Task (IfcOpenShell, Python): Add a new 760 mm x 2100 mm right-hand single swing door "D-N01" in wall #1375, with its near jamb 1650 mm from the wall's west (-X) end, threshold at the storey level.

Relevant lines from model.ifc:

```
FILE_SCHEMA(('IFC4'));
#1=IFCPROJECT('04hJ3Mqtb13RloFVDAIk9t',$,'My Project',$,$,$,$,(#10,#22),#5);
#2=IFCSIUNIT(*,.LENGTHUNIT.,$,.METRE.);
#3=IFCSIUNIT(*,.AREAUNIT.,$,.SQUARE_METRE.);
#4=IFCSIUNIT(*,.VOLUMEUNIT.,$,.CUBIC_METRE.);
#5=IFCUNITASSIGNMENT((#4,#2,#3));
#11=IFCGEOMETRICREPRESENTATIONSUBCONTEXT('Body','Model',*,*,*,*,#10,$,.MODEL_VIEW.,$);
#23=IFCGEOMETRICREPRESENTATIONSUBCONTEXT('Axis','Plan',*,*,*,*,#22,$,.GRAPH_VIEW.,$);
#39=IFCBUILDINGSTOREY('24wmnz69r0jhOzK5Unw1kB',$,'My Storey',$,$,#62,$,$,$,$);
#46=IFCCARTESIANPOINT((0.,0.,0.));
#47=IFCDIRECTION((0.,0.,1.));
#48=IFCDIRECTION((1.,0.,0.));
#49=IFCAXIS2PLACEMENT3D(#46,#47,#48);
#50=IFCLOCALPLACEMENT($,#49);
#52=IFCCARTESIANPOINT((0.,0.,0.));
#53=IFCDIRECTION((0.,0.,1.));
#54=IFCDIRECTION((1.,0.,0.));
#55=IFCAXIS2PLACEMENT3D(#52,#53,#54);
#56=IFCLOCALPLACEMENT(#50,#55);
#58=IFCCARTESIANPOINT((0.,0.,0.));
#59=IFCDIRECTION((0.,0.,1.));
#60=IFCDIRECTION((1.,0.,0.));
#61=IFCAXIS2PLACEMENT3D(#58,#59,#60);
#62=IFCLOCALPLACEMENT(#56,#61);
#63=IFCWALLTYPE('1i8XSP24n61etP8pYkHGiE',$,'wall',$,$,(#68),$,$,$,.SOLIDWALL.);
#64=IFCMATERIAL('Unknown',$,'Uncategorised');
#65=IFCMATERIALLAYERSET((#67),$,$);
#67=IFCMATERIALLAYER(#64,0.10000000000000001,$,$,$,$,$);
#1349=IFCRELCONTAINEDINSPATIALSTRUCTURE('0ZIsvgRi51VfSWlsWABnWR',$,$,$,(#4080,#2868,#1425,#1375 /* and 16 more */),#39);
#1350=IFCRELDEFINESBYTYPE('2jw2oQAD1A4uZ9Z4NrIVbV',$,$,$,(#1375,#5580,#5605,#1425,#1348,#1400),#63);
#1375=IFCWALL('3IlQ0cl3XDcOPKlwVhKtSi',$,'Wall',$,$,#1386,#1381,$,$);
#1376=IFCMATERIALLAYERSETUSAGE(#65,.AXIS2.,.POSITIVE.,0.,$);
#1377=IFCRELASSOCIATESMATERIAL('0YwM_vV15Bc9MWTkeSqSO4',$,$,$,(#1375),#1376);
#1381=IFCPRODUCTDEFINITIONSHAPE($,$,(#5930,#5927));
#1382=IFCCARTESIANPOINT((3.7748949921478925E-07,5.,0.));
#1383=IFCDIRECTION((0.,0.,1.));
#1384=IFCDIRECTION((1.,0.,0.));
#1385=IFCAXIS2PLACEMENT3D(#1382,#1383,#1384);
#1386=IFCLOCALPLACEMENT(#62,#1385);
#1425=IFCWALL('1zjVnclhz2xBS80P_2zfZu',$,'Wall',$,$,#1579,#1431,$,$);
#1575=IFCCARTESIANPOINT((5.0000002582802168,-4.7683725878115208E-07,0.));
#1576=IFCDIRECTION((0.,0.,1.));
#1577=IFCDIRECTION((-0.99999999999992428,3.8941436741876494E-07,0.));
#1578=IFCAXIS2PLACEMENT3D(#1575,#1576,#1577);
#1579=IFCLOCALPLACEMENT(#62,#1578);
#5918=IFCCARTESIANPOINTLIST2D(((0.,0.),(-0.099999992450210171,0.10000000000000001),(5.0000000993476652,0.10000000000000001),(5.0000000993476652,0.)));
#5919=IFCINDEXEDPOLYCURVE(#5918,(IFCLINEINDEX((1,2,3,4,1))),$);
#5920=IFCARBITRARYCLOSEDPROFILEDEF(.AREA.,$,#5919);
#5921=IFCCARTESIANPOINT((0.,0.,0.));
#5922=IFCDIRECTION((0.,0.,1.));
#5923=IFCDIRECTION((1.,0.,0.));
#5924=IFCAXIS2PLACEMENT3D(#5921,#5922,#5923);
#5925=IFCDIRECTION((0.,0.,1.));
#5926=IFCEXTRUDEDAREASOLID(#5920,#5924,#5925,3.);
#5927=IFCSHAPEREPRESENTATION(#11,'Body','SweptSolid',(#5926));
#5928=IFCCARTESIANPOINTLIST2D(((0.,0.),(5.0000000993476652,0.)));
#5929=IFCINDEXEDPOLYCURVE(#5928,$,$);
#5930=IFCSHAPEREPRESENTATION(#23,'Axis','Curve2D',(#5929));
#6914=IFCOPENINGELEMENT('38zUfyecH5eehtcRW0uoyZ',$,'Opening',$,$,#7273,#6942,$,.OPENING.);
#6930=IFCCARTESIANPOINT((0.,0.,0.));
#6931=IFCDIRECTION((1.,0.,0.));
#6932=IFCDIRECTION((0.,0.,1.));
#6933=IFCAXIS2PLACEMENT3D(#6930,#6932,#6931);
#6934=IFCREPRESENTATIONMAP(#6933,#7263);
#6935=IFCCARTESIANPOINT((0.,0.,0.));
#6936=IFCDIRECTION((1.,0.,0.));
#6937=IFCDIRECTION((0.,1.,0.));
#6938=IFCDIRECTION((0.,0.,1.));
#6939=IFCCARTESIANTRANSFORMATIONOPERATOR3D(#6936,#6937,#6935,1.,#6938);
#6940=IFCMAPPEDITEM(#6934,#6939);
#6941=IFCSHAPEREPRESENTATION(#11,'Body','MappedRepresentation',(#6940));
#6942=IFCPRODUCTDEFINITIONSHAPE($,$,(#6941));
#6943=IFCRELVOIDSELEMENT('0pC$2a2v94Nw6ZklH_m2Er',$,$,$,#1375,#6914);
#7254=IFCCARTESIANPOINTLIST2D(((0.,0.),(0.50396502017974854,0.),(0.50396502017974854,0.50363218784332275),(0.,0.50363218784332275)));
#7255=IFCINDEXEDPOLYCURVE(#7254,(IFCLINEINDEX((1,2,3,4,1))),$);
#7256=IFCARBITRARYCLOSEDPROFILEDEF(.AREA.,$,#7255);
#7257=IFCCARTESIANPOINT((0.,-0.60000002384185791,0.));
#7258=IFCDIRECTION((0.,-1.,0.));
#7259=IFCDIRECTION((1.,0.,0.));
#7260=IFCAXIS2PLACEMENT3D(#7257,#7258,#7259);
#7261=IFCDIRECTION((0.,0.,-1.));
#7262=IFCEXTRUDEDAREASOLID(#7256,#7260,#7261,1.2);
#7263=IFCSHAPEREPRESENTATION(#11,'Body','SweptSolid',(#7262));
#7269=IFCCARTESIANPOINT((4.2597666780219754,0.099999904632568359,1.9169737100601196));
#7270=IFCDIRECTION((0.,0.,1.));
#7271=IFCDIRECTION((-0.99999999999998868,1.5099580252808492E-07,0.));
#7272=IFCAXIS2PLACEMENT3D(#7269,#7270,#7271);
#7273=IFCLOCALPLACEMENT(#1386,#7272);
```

```python
import numpy as np
import ifcopenshell
import ifcopenshell.api.feature
import ifcopenshell.api.geometry
import ifcopenshell.api.root
import ifcopenshell.api.spatial
import ifcopenshell.geom
import ifcopenshell.util.element
import ifcopenshell.util.placement
import ifcopenshell.util.representation
import ifcopenshell.util.shape
import ifcopenshell.util.unit

model = ifcopenshell.open("model.ifc")
unit_scale = ifcopenshell.util.unit.calculate_unit_scale(model)
settings = ifcopenshell.geom.settings()


def volume(element):
    """Net volume in cubic metres, openings subtracted."""
    shape = ifcopenshell.geom.create_shape(settings, element)
    return ifcopenshell.util.shape.get_volume(shape.geometry)


wall = model.by_guid("3IlQ0cl3XDcOPKlwVhKtSi")
storey = ifcopenshell.util.element.get_container(wall, ifc_class="IfcBuildingStorey")
context = ifcopenshell.util.representation.get_context(model, "Model", "Body", "MODEL_VIEW")
before = volume(wall)

width, height, from_end, sill = 0.76, 2.1, 1.65, 0.0  # metres

# The wall runs along its own X axis, and the end named is its -X end.
wall_shape = ifcopenshell.geom.create_shape(settings, wall)
x, y, z = ifcopenshell.util.shape.get_vertices(wall_shape.geometry).T
start = x.min() + from_end
face, thickness = float(y.min()), float(y.max() - y.min())
wall_matrix = ifcopenshell.util.placement.get_local_placement(wall.ObjectPlacement)
level = ifcopenshell.util.placement.get_local_placement(storey.ObjectPlacement)[2, 3]


def in_wall(x, y):
    """Placement at x, y metres in the wall's axes, at sill height."""
    matrix = wall_matrix.copy()
    matrix[:, 3] = wall_matrix @ np.array([x / unit_scale, y / unit_scale, 0.0, 1.0])
    matrix[2, 3] = level + sill / unit_scale
    return matrix


# Opening: a box that overshoots both wall faces by 50 mm.
opening = ifcopenshell.api.root.create_entity(model, ifc_class="IfcOpeningElement", predefined_type="OPENING")
box = ifcopenshell.api.geometry.add_wall_representation(
    model, context=context, length=width, height=height, thickness=thickness + 0.1
)
ifcopenshell.api.geometry.assign_representation(model, product=opening, representation=box)
ifcopenshell.api.geometry.edit_object_placement(model, product=opening, matrix=in_wall(start, face - 0.05), is_si=False)
ifcopenshell.api.feature.add_feature(model, feature=opening, element=wall)

door = ifcopenshell.api.root.create_entity(model, ifc_class="IfcDoor", name="D-N01", predefined_type="DOOR")
door.OverallWidth, door.OverallHeight = width / unit_scale, height / unit_scale
door.OperationType = "SINGLE_SWING_RIGHT"
body = ifcopenshell.api.geometry.add_door_representation(
    model,
    context=context,
    overall_width=door.OverallWidth,
    overall_height=door.OverallHeight,
    operation_type="SINGLE_SWING_RIGHT",
    lining_properties={"LiningDepth": thickness / unit_scale, "ThresholdDepth": thickness / unit_scale},
)
ifcopenshell.api.geometry.assign_representation(model, product=door, representation=body)
ifcopenshell.api.spatial.assign_container(model, products=[door], relating_structure=storey)
ifcopenshell.api.feature.add_filling(model, opening=opening, element=door)

# The lining spans the wall, so the door starts at the wall face.
ifcopenshell.api.geometry.edit_object_placement(model, product=door, matrix=in_wall(start, face), is_si=False)

after = volume(wall)

print(f"wall volume {before:.3f} -> {after:.3f} m3")

model.write("model_updated.ifc")
```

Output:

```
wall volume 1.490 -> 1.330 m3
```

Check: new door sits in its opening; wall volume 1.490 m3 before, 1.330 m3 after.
